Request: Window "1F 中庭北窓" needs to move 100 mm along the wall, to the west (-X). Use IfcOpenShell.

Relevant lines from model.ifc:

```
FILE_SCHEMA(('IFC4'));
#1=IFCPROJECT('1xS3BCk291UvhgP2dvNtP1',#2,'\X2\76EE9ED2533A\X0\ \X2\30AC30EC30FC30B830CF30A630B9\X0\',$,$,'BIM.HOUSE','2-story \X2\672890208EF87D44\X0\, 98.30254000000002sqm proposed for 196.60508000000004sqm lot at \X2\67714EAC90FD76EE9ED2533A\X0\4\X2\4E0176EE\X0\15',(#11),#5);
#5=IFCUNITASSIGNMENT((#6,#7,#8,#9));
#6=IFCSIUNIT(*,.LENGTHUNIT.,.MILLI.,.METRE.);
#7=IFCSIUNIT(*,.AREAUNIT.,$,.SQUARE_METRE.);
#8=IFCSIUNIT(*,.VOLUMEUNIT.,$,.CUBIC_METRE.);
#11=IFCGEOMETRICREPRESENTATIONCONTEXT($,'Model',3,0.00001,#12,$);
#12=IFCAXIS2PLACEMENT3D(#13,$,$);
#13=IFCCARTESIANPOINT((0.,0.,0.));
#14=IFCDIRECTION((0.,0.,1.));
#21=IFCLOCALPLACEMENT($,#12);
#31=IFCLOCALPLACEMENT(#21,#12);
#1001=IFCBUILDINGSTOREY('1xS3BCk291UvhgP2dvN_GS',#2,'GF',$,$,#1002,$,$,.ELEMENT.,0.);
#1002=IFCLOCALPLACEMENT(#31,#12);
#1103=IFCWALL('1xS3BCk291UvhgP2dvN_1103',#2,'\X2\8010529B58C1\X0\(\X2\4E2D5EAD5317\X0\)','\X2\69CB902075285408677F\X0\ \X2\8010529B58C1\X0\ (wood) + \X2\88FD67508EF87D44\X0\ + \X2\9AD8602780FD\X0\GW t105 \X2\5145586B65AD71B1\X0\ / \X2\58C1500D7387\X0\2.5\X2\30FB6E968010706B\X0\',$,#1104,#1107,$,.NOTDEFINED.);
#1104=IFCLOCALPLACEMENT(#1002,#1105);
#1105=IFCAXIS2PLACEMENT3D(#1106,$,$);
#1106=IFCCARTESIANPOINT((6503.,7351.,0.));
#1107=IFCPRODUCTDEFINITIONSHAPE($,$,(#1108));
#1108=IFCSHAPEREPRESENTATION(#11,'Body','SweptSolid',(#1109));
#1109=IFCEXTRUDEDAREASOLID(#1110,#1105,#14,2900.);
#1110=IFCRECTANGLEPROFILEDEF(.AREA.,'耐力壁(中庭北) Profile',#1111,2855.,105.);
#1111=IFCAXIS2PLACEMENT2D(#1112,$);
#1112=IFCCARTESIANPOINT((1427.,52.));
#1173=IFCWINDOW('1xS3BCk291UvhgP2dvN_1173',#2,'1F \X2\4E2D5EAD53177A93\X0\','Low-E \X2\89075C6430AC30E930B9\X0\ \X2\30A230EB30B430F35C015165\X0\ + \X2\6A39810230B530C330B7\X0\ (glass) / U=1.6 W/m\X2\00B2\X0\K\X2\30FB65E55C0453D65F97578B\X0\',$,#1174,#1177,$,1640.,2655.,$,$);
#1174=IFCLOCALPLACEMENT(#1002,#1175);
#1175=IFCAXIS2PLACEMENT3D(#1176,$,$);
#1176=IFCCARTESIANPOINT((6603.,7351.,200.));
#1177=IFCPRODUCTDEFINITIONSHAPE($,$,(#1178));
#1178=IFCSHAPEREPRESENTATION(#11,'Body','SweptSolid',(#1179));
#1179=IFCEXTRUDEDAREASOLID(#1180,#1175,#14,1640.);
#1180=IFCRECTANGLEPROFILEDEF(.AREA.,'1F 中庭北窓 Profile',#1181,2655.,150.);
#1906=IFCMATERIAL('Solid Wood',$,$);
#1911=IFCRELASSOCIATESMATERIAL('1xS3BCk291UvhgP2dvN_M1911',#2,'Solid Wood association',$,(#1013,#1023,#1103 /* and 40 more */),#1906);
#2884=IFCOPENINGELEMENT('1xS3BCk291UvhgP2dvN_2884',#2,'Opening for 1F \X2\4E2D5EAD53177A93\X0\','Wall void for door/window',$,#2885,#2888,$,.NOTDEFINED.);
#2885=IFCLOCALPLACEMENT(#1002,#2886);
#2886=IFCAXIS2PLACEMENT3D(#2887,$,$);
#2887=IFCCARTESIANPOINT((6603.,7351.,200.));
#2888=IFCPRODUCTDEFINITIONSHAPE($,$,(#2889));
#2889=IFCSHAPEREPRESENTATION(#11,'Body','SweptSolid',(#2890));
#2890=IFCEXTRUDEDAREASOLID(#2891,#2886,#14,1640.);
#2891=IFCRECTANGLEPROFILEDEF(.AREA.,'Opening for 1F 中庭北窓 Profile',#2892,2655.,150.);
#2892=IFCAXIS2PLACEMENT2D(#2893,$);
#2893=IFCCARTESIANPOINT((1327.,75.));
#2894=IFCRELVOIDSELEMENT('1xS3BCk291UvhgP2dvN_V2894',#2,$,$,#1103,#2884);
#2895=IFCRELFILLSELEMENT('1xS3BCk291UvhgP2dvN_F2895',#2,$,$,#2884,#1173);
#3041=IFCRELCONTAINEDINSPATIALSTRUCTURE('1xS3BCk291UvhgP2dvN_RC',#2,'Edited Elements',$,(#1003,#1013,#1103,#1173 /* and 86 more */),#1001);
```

```python
import ifcopenshell
import ifcopenshell.api.geometry
import ifcopenshell.util.placement
import ifcopenshell.util.unit

model = ifcopenshell.open("model.ifc")
unit_scale = ifcopenshell.util.unit.calculate_unit_scale(model)

window = model.by_guid("1xS3BCk291UvhgP2dvN_1173")
opening = window.FillsVoids[0].RelatingOpeningElement
wall = opening.VoidsElements[0].RelatingBuildingElement

wall_matrix = ifcopenshell.util.placement.get_local_placement(wall.ObjectPlacement)
shift = wall_matrix[:3, 0] * -0.1 / unit_scale
before = ifcopenshell.util.placement.get_local_placement(window.ObjectPlacement)[:3, 3].copy()

# The window is not placed relative to its opening, so move both.
for product in (opening, window):
    matrix = ifcopenshell.util.placement.get_local_placement(product.ObjectPlacement)
    matrix[:3, 3] += shift
    ifcopenshell.api.geometry.edit_object_placement(model, product=product, matrix=matrix, is_si=False)

after = ifcopenshell.util.placement.get_local_placement(window.ObjectPlacement)[:3, 3]
print("window moved by", (after - before).round(3) + 0.0)

model.write("model_updated.ifc")
```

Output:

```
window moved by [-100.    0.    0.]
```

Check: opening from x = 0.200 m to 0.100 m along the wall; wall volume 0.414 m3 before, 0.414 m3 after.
